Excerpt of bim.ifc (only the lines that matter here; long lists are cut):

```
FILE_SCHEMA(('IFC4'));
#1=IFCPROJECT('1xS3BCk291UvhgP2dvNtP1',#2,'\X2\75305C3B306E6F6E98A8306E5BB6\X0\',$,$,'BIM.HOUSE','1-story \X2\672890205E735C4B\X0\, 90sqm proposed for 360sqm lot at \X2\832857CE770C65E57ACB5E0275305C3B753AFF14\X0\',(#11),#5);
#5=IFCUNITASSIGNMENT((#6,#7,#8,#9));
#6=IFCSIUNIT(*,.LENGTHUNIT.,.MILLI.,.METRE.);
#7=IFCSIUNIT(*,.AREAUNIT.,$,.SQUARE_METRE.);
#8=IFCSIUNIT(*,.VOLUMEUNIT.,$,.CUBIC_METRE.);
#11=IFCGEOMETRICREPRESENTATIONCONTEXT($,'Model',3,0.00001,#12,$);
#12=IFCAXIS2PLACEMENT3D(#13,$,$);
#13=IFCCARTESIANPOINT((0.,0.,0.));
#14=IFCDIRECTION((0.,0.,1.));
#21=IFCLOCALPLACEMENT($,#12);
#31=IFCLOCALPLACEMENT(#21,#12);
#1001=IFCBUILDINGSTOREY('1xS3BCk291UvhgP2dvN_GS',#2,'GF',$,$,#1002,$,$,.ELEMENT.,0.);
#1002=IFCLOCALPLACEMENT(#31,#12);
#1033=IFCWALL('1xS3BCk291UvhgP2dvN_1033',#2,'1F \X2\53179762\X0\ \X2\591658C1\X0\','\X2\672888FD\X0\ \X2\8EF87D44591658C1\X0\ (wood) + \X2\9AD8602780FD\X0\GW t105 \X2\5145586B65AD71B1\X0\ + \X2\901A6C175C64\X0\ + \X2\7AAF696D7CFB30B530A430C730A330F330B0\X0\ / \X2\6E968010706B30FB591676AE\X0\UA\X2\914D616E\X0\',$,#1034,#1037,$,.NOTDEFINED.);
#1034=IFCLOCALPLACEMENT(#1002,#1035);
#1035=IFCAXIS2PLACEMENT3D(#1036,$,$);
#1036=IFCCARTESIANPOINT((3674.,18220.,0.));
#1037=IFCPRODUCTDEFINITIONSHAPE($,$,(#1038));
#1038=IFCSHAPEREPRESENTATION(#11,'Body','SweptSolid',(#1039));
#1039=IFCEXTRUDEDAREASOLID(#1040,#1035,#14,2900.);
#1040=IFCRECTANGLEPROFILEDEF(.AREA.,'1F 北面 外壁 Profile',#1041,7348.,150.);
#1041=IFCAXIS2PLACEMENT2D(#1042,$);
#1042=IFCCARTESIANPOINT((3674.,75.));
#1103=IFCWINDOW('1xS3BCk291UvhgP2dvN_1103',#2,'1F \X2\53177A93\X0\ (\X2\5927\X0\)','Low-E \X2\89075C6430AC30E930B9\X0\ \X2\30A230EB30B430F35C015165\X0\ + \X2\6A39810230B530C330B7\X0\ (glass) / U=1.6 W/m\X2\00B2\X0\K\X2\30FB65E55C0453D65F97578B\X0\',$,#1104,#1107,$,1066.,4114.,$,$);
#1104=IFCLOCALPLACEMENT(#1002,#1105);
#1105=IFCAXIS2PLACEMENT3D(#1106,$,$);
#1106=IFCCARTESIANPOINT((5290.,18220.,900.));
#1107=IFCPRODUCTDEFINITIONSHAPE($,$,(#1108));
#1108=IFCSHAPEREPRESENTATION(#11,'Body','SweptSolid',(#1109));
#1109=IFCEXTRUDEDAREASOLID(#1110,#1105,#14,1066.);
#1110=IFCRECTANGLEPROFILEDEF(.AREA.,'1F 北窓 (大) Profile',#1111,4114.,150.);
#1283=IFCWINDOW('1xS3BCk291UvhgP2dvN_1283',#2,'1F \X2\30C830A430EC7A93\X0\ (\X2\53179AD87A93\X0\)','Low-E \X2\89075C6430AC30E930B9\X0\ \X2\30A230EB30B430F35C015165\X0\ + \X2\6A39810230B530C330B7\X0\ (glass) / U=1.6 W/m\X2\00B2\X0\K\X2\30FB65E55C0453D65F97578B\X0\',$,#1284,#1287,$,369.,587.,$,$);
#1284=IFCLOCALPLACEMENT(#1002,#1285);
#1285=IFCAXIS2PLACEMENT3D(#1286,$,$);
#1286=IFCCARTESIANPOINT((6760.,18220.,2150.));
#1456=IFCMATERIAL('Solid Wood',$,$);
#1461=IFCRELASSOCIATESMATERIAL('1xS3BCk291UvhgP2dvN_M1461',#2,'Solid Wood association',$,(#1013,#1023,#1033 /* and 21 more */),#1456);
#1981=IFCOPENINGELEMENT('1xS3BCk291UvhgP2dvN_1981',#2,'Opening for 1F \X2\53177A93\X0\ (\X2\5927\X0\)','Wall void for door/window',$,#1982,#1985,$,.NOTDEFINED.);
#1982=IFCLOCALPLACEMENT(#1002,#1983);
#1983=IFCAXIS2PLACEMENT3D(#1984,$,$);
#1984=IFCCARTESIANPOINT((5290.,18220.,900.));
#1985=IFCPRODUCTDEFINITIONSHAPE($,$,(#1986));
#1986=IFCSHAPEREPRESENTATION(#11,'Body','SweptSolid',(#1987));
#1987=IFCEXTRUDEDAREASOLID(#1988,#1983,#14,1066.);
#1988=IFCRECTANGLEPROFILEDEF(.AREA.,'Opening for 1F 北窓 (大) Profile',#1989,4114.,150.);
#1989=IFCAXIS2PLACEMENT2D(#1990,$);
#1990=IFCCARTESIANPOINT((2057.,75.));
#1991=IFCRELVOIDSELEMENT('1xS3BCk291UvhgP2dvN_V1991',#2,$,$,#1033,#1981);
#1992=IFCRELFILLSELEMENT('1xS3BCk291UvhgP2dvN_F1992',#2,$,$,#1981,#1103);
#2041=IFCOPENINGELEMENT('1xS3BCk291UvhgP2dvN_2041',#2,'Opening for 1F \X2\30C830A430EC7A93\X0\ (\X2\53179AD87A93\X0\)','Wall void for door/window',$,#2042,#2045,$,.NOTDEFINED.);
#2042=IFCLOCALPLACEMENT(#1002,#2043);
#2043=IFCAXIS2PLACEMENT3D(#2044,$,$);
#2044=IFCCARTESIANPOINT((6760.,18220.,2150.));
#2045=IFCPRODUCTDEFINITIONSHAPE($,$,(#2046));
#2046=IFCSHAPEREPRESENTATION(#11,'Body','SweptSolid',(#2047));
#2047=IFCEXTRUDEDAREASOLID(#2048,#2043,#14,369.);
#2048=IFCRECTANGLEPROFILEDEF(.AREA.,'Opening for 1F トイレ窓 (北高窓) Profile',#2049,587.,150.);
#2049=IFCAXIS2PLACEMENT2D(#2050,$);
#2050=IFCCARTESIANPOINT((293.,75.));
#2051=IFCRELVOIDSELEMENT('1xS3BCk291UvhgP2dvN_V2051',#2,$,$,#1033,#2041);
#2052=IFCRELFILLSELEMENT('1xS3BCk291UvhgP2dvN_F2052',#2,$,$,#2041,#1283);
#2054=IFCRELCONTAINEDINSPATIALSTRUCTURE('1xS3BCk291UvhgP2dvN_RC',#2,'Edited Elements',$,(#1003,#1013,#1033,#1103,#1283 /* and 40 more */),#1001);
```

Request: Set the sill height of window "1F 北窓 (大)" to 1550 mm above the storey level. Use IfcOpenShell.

```python
import numpy as np
import ifcopenshell
import ifcopenshell.api.geometry
import ifcopenshell.geom
import ifcopenshell.util.element
import ifcopenshell.util.placement
import ifcopenshell.util.shape
import ifcopenshell.util.unit

model = ifcopenshell.open("bim.ifc")
unit_scale = ifcopenshell.util.unit.calculate_unit_scale(model)

window = model.by_id(1103)
opening = window.FillsVoids[0].RelatingOpeningElement
storey = ifcopenshell.util.element.get_container(window, ifc_class="IfcBuildingStorey")
level = ifcopenshell.util.placement.get_local_placement(storey.ObjectPlacement)[2, 3]

# The opening's origin need not be at the sill, so measure its lowest point.
shape = ifcopenshell.geom.create_shape(ifcopenshell.geom.settings(), opening)
bottom = ifcopenshell.util.shape.get_shape_bottom_elevation(shape, shape.geometry) / unit_scale
dz = level + 1.55 / unit_scale - bottom

shift = np.array([0.0, 0.0, dz])
# The window is not placed relative to its opening, so move both.
for product in (opening, window):
    matrix = ifcopenshell.util.placement.get_local_placement(product.ObjectPlacement)
    matrix[:3, 3] += shift
    ifcopenshell.api.geometry.edit_object_placement(model, product=product, matrix=matrix, is_si=False)

print(f"moved by {dz * unit_scale:+.3f} m")

model.write("bim_edited.ifc")
```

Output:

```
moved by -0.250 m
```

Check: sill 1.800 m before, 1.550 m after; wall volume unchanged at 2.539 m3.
